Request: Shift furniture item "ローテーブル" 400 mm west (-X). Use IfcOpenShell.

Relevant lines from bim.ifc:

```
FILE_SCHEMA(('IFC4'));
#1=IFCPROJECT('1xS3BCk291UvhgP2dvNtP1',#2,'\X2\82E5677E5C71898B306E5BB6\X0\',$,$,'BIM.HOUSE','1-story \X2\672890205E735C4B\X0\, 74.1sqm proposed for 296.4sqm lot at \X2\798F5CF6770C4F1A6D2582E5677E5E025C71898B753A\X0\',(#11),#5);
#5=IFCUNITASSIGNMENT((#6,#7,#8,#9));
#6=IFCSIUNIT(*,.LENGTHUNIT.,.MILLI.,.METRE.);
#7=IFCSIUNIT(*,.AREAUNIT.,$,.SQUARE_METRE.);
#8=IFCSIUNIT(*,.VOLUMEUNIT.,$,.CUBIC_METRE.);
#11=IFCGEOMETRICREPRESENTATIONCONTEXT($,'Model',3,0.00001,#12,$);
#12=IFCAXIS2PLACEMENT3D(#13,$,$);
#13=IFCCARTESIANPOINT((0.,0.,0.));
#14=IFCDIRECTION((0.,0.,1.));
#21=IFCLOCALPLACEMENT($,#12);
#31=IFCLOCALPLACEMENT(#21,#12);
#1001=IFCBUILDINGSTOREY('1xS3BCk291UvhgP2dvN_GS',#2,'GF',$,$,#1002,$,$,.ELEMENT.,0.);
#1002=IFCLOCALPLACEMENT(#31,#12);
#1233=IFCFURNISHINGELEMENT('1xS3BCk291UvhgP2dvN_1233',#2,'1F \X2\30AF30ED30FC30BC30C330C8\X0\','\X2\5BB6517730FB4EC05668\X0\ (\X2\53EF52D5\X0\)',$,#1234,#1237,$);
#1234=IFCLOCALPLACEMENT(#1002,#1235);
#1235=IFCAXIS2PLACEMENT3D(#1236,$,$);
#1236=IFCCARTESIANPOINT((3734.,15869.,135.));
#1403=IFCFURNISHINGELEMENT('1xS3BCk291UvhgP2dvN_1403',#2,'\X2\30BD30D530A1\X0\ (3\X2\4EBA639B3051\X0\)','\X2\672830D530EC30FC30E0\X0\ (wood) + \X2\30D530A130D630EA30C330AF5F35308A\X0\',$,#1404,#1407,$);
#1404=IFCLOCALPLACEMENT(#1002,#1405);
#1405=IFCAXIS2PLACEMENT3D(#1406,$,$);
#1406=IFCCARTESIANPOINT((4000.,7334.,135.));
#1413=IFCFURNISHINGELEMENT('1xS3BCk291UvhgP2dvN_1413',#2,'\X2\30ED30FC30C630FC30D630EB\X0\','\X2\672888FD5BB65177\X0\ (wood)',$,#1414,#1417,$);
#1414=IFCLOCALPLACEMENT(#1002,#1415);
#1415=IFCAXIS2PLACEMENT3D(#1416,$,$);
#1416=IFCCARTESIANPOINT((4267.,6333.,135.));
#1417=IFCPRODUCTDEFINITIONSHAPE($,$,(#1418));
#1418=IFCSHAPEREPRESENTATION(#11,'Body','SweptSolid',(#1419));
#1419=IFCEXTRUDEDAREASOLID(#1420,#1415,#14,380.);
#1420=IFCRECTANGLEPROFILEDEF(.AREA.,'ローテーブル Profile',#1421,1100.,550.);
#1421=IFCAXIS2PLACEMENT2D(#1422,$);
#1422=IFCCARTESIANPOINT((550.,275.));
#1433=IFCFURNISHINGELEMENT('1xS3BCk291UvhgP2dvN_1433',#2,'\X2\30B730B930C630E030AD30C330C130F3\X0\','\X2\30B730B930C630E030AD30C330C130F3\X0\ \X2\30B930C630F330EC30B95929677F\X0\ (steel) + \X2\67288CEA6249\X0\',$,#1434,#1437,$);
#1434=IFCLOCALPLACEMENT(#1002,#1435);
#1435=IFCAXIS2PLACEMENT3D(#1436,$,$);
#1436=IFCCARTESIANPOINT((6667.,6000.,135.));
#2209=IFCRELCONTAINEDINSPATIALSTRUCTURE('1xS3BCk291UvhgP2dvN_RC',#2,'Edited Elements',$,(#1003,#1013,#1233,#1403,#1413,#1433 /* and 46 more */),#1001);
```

```python
import ifcopenshell
import ifcopenshell.api.geometry
import ifcopenshell.util.placement

model = ifcopenshell.open("bim.ifc")

item = model.by_guid("1xS3BCk291UvhgP2dvN_1413")
matrix = ifcopenshell.util.placement.get_local_placement(item.ObjectPlacement)
matrix[0, 3] -= 400.0
ifcopenshell.api.geometry.edit_object_placement(model, product=item, matrix=matrix, is_si=False)

print(ifcopenshell.util.placement.get_local_placement(item.ObjectPlacement).round(3) + 0.0)

model.write("bim_rev.ifc")
```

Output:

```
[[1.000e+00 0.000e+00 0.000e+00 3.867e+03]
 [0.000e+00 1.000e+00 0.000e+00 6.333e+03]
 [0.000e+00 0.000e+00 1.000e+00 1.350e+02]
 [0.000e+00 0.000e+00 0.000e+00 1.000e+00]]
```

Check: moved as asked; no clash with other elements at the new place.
